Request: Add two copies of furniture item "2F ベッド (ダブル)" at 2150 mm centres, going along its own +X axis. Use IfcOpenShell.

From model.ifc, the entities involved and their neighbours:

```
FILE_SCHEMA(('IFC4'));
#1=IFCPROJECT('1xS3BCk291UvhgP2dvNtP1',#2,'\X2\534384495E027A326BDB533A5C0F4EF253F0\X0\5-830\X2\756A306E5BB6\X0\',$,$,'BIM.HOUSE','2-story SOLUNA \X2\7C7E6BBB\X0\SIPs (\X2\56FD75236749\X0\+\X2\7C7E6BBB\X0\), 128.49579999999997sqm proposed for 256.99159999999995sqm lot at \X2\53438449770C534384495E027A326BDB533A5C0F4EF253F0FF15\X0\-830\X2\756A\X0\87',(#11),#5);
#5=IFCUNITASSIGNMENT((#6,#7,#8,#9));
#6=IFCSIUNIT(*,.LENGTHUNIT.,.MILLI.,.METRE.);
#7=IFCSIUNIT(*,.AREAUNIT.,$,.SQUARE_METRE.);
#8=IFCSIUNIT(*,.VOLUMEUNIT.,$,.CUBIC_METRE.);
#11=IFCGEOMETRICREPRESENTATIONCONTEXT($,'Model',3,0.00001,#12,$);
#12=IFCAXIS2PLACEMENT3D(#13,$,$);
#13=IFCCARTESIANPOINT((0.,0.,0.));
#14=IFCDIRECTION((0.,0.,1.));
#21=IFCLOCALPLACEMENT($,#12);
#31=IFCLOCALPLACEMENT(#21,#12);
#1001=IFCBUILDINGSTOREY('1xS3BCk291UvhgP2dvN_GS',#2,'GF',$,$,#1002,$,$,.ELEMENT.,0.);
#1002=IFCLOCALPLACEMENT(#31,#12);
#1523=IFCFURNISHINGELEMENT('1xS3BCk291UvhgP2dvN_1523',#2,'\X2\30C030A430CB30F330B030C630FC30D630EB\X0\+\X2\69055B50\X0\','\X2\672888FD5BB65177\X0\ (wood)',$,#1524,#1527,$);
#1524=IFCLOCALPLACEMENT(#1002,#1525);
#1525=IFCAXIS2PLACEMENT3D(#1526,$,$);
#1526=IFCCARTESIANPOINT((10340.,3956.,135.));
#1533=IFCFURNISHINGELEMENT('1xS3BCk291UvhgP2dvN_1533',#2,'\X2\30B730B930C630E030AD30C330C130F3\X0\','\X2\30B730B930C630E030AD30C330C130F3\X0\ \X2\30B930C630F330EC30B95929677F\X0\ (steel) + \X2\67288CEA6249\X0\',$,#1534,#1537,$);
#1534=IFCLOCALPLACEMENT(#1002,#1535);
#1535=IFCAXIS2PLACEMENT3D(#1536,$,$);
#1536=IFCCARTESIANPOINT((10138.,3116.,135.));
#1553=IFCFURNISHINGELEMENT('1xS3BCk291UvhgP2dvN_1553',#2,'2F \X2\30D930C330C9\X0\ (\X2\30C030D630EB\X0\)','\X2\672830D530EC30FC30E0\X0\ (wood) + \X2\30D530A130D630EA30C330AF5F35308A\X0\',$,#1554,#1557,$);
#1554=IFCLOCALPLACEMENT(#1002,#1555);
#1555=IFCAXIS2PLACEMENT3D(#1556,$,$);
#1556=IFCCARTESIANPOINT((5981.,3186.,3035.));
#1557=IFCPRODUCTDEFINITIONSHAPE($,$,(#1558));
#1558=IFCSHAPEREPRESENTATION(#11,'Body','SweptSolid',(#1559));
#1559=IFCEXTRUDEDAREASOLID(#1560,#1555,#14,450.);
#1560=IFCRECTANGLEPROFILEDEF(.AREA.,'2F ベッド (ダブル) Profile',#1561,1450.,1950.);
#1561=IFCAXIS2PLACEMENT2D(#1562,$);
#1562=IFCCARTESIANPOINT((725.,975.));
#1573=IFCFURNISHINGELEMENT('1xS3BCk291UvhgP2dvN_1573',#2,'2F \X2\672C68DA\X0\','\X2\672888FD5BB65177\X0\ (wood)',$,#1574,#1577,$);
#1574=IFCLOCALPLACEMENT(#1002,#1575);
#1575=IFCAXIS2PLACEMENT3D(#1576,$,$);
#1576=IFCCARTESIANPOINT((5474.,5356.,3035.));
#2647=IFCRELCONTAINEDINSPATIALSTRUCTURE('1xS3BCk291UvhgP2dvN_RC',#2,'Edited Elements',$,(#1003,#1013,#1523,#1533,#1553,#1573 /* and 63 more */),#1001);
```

```python
import ifcopenshell
import ifcopenshell.api.geometry
import ifcopenshell.api.root
import ifcopenshell.util.element
import ifcopenshell.util.placement
import ifcopenshell.util.unit

model = ifcopenshell.open("model.ifc")
unit_scale = ifcopenshell.util.unit.calculate_unit_scale(model)


def reuse_history(source, copy):
    """copy_class also copies each property set's owner history, people and application; keep the originals."""
    for rel in copy.IsDefinedBy:
        if rel.is_a("IfcRelDefinesByProperties") and (history := rel.RelatingPropertyDefinition.OwnerHistory):
            rel.RelatingPropertyDefinition.OwnerHistory = source.OwnerHistory
            ifcopenshell.util.element.remove_deep2(model, history)


source = model.by_guid("1xS3BCk291UvhgP2dvN_1553")
base = ifcopenshell.util.placement.get_local_placement(source.ObjectPlacement)
step = base[:3, 0] * 2.15 / unit_scale

for i in range(1, 3):
    copy = ifcopenshell.api.root.copy_class(model, product=source)
    copy.Representation = ifcopenshell.util.element.copy_deep(
        model, source.Representation, exclude=["IfcGeometricRepresentationContext", "IfcRepresentationMap"]
    )
    reuse_history(source, copy)
    matrix = base.copy()
    matrix[:3, 3] += i * step
    print("added at", matrix[:3, 3].round(3) + 0.0)
    ifcopenshell.api.geometry.edit_object_placement(model, product=copy, matrix=matrix, is_si=False)

model.write("model_rev.ifc")
```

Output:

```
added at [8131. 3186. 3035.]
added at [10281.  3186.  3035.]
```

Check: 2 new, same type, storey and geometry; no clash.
